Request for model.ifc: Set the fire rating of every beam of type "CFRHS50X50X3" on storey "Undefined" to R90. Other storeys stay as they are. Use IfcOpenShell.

First a look at what the model holds.

```python
import ifcopenshell
import ifcopenshell.util.element

model = ifcopenshell.open("model.ifc")
print(model.schema)
storey = next(s for s in model.by_type("IfcBuildingStorey") if s.Name == "Undefined")
beams = [e for e in ifcopenshell.util.element.get_decomposition(storey) if e.is_a("IfcBeam")]
seen = {}
for e in beams:
    element_type = ifcopenshell.util.element.get_type(e)
    key = (element_type.Name if element_type != e and element_type else None, ifcopenshell.util.element.get_pset(e, "Pset_BeamCommon", "FireRating"))
    seen[key] = seen.get(key, 0) + 1
for (name, value), count in sorted(seen.items(), key=str):
    print(count, "x", name, "|", value)
```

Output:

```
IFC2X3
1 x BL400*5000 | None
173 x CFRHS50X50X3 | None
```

```python
import ifcopenshell
import ifcopenshell.api.pset
import ifcopenshell.util.element

model = ifcopenshell.open("model.ifc")

storey = next(s for s in model.by_type("IfcBuildingStorey") if s.Name == "Undefined")
beams = [e for e in ifcopenshell.util.element.get_decomposition(storey) if e.is_a("IfcBeam")]

count = 0
for e in beams:
    element_type = ifcopenshell.util.element.get_type(e)
    if element_type in (None, e) or element_type.Name != "CFRHS50X50X3":
        continue
    found = ifcopenshell.util.element.get_pset(e, "Pset_BeamCommon", should_inherit=False)
    if found:
        pset = model.by_id(found["id"])
        if len(ifcopenshell.util.element.get_elements_by_pset(pset)) > 1:
            pset = ifcopenshell.api.pset.unshare_pset(model, products=[e], pset=pset)[0]
    else:
        pset = ifcopenshell.api.pset.add_pset(model, product=e, name="Pset_BeamCommon")
    ifcopenshell.api.pset.edit_pset(model, pset=pset, properties={"FireRating": "R90"})
    count += 1

print(count, "beams updated")

model.write("model_edited.ifc")
```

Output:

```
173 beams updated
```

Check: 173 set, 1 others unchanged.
